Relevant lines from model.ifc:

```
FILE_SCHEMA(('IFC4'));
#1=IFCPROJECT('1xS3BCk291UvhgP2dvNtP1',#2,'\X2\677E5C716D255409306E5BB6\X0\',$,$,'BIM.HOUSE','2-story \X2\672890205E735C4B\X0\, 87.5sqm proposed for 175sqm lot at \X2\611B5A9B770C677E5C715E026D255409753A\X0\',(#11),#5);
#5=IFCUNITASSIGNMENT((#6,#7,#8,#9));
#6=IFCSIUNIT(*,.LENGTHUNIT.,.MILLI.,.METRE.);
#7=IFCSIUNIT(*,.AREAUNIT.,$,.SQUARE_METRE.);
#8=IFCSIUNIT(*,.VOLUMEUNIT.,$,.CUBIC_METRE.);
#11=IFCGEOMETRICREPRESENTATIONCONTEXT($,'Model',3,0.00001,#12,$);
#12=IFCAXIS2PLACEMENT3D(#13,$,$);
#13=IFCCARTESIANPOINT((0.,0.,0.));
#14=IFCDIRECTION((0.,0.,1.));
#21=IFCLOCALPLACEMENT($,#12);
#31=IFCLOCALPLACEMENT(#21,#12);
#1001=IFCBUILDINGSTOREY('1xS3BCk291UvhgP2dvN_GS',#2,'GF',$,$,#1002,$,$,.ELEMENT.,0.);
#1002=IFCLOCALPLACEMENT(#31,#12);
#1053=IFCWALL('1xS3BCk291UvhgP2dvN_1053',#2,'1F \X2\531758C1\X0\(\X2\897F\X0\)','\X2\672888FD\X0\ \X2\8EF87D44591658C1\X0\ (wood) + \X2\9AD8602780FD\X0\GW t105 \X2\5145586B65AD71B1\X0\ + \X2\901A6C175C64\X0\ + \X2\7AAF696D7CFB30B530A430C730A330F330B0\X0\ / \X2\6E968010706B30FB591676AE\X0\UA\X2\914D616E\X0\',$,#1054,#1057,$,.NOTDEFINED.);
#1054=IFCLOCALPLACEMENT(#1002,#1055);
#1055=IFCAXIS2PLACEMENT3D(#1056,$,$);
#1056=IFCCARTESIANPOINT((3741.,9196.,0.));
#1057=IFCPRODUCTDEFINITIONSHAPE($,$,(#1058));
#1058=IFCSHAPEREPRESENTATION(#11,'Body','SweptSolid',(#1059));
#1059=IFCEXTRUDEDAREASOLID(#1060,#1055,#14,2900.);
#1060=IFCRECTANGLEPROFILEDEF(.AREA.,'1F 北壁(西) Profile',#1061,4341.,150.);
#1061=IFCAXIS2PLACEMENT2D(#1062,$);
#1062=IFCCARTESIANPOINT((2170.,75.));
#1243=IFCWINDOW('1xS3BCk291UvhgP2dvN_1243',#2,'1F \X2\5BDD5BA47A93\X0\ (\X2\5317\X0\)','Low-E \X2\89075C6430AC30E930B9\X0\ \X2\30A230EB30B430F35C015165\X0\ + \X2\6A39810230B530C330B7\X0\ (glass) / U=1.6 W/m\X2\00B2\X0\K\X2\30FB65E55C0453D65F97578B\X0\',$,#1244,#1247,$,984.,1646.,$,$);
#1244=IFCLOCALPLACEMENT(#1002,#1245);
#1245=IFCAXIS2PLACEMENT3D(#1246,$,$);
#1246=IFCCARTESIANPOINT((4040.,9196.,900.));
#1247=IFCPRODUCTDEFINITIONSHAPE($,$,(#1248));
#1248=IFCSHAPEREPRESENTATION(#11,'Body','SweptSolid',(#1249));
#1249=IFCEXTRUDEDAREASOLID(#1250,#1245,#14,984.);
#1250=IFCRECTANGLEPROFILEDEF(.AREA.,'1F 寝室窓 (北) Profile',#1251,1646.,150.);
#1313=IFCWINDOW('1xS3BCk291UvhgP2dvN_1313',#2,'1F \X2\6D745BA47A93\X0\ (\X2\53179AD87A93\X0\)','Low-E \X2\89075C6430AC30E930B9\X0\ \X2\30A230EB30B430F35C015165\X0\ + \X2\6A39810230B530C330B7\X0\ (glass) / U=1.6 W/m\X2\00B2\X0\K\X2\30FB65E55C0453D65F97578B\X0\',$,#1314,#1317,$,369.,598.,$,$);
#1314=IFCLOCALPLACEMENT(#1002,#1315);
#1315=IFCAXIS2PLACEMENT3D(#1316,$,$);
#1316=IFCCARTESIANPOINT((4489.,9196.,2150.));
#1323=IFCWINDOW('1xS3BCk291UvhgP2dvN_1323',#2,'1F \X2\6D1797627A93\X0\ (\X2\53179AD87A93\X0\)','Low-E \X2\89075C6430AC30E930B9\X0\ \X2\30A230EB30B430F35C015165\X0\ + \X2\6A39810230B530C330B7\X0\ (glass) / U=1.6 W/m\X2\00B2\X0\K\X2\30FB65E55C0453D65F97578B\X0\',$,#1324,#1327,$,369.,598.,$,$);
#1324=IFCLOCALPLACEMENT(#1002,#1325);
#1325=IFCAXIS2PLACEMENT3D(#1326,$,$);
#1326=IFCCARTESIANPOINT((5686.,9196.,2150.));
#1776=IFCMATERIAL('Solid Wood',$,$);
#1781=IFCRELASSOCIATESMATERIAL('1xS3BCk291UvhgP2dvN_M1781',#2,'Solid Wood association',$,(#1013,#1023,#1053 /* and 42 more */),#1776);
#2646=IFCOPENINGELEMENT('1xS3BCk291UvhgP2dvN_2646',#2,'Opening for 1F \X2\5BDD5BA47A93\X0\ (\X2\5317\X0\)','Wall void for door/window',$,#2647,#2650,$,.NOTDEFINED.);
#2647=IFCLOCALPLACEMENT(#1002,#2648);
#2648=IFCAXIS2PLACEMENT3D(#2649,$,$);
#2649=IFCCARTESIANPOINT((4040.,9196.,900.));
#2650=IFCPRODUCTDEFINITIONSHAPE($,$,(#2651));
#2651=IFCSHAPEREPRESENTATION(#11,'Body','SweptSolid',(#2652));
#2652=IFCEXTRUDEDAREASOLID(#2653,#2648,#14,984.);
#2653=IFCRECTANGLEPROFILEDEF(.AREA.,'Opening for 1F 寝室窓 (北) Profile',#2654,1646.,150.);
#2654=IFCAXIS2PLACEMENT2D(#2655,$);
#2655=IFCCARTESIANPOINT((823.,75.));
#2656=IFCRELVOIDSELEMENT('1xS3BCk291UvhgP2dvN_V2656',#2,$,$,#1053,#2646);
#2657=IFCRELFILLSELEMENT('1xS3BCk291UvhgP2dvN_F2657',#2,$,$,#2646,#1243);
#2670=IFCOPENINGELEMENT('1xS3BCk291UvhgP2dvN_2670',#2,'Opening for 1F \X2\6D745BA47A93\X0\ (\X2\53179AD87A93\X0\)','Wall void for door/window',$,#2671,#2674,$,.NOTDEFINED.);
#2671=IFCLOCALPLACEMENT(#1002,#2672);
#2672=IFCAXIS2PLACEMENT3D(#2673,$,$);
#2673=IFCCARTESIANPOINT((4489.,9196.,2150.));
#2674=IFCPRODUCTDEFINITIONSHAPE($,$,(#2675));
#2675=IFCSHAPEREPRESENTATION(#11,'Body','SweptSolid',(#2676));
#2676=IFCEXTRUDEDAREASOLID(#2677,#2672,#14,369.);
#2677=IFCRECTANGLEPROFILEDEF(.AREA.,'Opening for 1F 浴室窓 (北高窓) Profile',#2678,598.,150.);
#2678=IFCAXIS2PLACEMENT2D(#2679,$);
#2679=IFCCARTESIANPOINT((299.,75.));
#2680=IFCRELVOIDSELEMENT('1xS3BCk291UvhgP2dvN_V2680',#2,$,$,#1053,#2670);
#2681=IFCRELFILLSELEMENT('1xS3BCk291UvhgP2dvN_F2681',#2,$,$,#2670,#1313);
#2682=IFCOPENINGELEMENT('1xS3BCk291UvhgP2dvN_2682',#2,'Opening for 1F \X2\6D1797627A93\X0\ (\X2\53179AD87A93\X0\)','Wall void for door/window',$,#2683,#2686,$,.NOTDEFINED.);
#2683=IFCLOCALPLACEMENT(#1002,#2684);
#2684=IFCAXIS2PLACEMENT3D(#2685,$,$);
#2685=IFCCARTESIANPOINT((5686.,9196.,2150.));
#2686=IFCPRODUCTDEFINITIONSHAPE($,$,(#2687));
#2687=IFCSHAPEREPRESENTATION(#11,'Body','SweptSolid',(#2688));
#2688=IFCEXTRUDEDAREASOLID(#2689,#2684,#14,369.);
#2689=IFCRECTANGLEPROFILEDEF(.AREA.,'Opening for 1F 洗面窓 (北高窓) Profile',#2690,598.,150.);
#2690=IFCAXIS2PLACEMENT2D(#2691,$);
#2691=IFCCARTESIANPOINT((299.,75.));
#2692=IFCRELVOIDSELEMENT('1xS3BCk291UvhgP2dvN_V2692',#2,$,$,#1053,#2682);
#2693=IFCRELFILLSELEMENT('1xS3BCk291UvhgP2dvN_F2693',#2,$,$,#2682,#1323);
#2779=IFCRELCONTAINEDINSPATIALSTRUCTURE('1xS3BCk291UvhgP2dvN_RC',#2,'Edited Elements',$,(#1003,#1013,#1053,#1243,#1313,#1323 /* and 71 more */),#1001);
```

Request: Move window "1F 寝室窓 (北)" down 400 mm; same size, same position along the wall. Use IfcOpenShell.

```python
import numpy as np
import ifcopenshell
import ifcopenshell.api.geometry
import ifcopenshell.util.placement
import ifcopenshell.util.unit

model = ifcopenshell.open("model.ifc")
unit_scale = ifcopenshell.util.unit.calculate_unit_scale(model)

window = model.by_id(1243)
opening = window.FillsVoids[0].RelatingOpeningElement
dz = -400.0

shift = np.array([0.0, 0.0, dz])
# The window is not placed relative to its opening, so move both.
for product in (opening, window):
    matrix = ifcopenshell.util.placement.get_local_placement(product.ObjectPlacement)
    matrix[:3, 3] += shift
    ifcopenshell.api.geometry.edit_object_placement(model, product=product, matrix=matrix, is_si=False)

print(f"moved by {dz * unit_scale:+.3f} m")

model.write("model-out.ifc")
```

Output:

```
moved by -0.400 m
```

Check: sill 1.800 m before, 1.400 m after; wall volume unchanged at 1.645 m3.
